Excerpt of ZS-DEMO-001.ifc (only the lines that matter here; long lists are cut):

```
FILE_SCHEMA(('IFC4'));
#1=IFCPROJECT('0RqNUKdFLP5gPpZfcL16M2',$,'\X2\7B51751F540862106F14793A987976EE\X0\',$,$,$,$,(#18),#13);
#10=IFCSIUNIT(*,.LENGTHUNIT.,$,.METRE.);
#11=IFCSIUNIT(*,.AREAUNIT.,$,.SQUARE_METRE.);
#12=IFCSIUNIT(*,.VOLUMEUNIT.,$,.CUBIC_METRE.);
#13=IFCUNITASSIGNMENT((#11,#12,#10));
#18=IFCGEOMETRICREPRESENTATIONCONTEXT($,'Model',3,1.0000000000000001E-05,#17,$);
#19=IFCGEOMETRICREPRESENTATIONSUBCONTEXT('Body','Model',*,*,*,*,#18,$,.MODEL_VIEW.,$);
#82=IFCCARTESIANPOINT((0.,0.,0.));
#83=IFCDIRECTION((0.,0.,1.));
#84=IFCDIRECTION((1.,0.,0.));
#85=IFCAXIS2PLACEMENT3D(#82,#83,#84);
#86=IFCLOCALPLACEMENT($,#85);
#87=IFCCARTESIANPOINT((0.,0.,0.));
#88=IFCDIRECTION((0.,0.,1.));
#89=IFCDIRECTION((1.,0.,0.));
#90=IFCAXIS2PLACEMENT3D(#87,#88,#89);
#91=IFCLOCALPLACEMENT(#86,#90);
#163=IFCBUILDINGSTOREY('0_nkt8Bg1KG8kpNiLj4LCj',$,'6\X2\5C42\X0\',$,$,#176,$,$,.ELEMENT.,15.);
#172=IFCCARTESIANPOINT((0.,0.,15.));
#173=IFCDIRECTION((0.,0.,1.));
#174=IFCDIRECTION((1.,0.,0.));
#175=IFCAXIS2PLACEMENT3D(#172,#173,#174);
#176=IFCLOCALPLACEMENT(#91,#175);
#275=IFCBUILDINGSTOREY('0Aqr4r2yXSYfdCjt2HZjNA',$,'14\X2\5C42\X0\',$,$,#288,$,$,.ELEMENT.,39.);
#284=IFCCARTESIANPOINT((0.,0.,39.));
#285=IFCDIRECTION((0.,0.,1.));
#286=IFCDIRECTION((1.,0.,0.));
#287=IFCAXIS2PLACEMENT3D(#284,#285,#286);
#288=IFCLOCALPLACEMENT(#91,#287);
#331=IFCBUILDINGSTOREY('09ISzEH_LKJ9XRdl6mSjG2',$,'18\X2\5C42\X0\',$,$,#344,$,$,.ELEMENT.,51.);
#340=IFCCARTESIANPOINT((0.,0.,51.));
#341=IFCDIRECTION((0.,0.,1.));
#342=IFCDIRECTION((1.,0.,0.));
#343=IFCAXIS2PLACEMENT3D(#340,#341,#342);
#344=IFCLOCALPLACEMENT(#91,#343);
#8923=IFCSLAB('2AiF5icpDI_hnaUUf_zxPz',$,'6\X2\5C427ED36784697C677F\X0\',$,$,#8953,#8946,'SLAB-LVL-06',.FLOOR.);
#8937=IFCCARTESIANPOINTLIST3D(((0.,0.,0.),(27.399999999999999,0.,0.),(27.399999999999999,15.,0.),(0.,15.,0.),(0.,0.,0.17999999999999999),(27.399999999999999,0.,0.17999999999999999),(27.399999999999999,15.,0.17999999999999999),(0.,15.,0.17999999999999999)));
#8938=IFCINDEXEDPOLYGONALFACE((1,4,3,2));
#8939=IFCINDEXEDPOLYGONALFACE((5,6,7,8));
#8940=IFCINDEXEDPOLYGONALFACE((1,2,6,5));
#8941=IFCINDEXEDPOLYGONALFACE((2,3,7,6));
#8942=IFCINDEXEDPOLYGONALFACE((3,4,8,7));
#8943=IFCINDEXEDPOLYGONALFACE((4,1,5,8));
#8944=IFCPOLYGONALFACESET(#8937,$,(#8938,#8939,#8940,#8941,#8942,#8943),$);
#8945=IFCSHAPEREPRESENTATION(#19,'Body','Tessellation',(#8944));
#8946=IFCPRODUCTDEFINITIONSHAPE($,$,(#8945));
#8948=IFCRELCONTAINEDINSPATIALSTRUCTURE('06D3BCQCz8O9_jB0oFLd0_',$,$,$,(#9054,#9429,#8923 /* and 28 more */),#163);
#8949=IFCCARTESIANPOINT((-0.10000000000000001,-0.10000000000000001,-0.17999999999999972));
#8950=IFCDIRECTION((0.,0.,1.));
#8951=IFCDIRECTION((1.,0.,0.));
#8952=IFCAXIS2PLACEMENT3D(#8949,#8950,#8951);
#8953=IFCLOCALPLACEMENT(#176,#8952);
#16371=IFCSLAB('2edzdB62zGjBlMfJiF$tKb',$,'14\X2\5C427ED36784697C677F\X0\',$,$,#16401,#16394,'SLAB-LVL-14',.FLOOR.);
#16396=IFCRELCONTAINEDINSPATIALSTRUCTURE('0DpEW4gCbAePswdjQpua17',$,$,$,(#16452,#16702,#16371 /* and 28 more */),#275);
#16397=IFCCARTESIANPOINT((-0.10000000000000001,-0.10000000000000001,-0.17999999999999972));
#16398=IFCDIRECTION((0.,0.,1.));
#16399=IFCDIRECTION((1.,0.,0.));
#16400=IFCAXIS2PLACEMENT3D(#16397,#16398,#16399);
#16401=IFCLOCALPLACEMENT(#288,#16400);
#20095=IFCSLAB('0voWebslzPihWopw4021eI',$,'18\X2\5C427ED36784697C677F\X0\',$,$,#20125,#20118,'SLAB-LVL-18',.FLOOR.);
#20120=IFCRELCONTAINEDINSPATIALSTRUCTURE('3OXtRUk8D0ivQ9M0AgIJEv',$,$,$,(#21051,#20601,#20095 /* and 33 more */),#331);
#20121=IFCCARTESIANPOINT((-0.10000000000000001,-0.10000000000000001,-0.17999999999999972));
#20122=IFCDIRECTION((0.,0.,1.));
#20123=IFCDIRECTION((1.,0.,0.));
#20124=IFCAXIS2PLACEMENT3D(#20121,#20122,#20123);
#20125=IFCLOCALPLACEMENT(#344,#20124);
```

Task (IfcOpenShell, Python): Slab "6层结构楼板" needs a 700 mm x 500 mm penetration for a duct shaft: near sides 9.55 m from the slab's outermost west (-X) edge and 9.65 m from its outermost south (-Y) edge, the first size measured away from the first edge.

```python
import numpy as np
import ifcopenshell
import ifcopenshell.api.feature
import ifcopenshell.api.geometry
import ifcopenshell.api.root
import ifcopenshell.geom
import ifcopenshell.util.placement
import ifcopenshell.util.representation
import ifcopenshell.util.shape
import ifcopenshell.util.unit

model = ifcopenshell.open("ZS-DEMO-001.ifc")
unit_scale = ifcopenshell.util.unit.calculate_unit_scale(model)
settings = ifcopenshell.geom.settings()


def volume(element):
    """Net volume in cubic metres, openings subtracted."""
    shape = ifcopenshell.geom.create_shape(settings, element)
    return ifcopenshell.util.shape.get_volume(shape.geometry)


slab = model.by_guid("2AiF5icpDI_hnaUUf_zxPz")
before = volume(slab)

# Extent in the slab's own axes, in metres. The edges named are its -X and -Y sides.
slab_shape = ifcopenshell.geom.create_shape(settings, slab)
vertices = ifcopenshell.util.shape.get_vertices(slab_shape.geometry)
x_min, y_min, bottom = vertices.min(axis=0)
top = vertices[:, 2].max()

opening = ifcopenshell.api.root.create_entity(model, ifc_class="IfcOpeningElement", name="Duct shaft opening", predefined_type="OPENING")
context = ifcopenshell.util.representation.get_context(model, "Model", "Body", "MODEL_VIEW")
width, depth = 0.7, 0.5
outline = [(0.0, 0.0), (width, 0.0), (width, depth), (0.0, depth), (0.0, 0.0)]
# Overshoot both faces by 50 mm so the cut is clean.
shape = ifcopenshell.api.geometry.add_slab_representation(
    model, context=context, depth=top - bottom + 0.1, polyline=outline
)
ifcopenshell.api.geometry.assign_representation(model, product=opening, representation=shape)

matrix = ifcopenshell.util.placement.get_local_placement(slab.ObjectPlacement)
matrix[:, 3] = matrix @ np.append(np.array([x_min + 9.55, y_min + 9.65, bottom - 0.05]) / unit_scale, 1.0)
ifcopenshell.api.geometry.edit_object_placement(model, product=opening, matrix=matrix, is_si=False)
ifcopenshell.api.feature.add_feature(model, feature=opening, element=slab)

after = volume(slab)

print(f"slab volume {before:.3f} -> {after:.3f} m3")

model.write("ZS-DEMO-001_rev.ifc")
```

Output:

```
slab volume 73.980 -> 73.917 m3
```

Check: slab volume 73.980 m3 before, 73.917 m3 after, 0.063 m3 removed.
